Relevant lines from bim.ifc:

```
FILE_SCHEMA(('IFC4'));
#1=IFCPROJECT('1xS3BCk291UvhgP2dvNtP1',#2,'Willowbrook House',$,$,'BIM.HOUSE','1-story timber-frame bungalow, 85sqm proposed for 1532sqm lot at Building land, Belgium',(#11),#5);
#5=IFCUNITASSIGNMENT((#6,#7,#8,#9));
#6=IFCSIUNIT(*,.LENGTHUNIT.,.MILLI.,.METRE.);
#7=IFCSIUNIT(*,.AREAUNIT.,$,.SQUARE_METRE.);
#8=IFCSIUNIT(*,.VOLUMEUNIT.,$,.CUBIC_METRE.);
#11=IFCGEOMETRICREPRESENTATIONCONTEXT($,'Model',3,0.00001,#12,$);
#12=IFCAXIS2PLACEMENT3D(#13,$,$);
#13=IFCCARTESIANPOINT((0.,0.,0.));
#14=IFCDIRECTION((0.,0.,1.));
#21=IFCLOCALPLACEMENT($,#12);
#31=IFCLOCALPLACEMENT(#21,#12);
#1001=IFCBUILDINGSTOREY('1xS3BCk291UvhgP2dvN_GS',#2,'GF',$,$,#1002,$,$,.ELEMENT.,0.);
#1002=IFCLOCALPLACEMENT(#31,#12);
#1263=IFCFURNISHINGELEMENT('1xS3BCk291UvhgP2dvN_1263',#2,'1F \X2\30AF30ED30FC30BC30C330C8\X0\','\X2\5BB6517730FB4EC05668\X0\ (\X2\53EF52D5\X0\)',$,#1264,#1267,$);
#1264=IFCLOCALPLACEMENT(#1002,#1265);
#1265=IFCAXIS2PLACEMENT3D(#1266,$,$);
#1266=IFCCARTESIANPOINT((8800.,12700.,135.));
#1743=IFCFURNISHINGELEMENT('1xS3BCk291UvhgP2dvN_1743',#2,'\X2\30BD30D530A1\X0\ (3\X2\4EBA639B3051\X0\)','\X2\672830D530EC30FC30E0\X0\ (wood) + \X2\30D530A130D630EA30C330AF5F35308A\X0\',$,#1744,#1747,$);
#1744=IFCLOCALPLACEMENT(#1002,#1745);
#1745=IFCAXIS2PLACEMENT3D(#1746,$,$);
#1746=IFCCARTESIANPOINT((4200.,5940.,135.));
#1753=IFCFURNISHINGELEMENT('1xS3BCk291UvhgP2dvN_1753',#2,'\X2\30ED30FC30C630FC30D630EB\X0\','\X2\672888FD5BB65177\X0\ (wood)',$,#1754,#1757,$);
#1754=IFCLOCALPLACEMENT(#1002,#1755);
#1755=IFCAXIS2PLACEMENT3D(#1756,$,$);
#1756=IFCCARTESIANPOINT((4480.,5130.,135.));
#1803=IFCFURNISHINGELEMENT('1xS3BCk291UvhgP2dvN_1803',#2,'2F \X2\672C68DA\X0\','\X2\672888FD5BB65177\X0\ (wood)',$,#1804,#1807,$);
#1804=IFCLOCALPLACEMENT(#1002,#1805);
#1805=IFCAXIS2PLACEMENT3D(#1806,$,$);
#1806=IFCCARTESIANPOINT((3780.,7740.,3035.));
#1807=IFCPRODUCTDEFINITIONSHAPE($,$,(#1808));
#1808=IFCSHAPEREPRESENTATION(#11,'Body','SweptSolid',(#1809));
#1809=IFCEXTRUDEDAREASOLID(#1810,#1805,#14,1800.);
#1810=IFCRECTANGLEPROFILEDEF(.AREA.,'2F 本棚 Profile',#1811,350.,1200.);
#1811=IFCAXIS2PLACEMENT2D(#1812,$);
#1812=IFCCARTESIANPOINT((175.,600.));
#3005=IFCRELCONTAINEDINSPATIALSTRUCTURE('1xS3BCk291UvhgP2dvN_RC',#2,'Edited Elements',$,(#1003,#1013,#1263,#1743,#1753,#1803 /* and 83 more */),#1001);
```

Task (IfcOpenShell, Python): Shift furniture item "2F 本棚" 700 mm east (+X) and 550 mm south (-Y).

```python
import ifcopenshell
import ifcopenshell.api.geometry
import ifcopenshell.util.placement
import ifcopenshell.util.unit

model = ifcopenshell.open("bim.ifc")
unit_scale = ifcopenshell.util.unit.calculate_unit_scale(model)

item = model.by_id(1803)
matrix = ifcopenshell.util.placement.get_local_placement(item.ObjectPlacement)
matrix[0, 3] += 0.7 / unit_scale
matrix[1, 3] -= 0.55 / unit_scale
ifcopenshell.api.geometry.edit_object_placement(model, product=item, matrix=matrix, is_si=False)

print(ifcopenshell.util.placement.get_local_placement(item.ObjectPlacement).round(3) + 0.0)

model.write("bim_edited.ifc")
```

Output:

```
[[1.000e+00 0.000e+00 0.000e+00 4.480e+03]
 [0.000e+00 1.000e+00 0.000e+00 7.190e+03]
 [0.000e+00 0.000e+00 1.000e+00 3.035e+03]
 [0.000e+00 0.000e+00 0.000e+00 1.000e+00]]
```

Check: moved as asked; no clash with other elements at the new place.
